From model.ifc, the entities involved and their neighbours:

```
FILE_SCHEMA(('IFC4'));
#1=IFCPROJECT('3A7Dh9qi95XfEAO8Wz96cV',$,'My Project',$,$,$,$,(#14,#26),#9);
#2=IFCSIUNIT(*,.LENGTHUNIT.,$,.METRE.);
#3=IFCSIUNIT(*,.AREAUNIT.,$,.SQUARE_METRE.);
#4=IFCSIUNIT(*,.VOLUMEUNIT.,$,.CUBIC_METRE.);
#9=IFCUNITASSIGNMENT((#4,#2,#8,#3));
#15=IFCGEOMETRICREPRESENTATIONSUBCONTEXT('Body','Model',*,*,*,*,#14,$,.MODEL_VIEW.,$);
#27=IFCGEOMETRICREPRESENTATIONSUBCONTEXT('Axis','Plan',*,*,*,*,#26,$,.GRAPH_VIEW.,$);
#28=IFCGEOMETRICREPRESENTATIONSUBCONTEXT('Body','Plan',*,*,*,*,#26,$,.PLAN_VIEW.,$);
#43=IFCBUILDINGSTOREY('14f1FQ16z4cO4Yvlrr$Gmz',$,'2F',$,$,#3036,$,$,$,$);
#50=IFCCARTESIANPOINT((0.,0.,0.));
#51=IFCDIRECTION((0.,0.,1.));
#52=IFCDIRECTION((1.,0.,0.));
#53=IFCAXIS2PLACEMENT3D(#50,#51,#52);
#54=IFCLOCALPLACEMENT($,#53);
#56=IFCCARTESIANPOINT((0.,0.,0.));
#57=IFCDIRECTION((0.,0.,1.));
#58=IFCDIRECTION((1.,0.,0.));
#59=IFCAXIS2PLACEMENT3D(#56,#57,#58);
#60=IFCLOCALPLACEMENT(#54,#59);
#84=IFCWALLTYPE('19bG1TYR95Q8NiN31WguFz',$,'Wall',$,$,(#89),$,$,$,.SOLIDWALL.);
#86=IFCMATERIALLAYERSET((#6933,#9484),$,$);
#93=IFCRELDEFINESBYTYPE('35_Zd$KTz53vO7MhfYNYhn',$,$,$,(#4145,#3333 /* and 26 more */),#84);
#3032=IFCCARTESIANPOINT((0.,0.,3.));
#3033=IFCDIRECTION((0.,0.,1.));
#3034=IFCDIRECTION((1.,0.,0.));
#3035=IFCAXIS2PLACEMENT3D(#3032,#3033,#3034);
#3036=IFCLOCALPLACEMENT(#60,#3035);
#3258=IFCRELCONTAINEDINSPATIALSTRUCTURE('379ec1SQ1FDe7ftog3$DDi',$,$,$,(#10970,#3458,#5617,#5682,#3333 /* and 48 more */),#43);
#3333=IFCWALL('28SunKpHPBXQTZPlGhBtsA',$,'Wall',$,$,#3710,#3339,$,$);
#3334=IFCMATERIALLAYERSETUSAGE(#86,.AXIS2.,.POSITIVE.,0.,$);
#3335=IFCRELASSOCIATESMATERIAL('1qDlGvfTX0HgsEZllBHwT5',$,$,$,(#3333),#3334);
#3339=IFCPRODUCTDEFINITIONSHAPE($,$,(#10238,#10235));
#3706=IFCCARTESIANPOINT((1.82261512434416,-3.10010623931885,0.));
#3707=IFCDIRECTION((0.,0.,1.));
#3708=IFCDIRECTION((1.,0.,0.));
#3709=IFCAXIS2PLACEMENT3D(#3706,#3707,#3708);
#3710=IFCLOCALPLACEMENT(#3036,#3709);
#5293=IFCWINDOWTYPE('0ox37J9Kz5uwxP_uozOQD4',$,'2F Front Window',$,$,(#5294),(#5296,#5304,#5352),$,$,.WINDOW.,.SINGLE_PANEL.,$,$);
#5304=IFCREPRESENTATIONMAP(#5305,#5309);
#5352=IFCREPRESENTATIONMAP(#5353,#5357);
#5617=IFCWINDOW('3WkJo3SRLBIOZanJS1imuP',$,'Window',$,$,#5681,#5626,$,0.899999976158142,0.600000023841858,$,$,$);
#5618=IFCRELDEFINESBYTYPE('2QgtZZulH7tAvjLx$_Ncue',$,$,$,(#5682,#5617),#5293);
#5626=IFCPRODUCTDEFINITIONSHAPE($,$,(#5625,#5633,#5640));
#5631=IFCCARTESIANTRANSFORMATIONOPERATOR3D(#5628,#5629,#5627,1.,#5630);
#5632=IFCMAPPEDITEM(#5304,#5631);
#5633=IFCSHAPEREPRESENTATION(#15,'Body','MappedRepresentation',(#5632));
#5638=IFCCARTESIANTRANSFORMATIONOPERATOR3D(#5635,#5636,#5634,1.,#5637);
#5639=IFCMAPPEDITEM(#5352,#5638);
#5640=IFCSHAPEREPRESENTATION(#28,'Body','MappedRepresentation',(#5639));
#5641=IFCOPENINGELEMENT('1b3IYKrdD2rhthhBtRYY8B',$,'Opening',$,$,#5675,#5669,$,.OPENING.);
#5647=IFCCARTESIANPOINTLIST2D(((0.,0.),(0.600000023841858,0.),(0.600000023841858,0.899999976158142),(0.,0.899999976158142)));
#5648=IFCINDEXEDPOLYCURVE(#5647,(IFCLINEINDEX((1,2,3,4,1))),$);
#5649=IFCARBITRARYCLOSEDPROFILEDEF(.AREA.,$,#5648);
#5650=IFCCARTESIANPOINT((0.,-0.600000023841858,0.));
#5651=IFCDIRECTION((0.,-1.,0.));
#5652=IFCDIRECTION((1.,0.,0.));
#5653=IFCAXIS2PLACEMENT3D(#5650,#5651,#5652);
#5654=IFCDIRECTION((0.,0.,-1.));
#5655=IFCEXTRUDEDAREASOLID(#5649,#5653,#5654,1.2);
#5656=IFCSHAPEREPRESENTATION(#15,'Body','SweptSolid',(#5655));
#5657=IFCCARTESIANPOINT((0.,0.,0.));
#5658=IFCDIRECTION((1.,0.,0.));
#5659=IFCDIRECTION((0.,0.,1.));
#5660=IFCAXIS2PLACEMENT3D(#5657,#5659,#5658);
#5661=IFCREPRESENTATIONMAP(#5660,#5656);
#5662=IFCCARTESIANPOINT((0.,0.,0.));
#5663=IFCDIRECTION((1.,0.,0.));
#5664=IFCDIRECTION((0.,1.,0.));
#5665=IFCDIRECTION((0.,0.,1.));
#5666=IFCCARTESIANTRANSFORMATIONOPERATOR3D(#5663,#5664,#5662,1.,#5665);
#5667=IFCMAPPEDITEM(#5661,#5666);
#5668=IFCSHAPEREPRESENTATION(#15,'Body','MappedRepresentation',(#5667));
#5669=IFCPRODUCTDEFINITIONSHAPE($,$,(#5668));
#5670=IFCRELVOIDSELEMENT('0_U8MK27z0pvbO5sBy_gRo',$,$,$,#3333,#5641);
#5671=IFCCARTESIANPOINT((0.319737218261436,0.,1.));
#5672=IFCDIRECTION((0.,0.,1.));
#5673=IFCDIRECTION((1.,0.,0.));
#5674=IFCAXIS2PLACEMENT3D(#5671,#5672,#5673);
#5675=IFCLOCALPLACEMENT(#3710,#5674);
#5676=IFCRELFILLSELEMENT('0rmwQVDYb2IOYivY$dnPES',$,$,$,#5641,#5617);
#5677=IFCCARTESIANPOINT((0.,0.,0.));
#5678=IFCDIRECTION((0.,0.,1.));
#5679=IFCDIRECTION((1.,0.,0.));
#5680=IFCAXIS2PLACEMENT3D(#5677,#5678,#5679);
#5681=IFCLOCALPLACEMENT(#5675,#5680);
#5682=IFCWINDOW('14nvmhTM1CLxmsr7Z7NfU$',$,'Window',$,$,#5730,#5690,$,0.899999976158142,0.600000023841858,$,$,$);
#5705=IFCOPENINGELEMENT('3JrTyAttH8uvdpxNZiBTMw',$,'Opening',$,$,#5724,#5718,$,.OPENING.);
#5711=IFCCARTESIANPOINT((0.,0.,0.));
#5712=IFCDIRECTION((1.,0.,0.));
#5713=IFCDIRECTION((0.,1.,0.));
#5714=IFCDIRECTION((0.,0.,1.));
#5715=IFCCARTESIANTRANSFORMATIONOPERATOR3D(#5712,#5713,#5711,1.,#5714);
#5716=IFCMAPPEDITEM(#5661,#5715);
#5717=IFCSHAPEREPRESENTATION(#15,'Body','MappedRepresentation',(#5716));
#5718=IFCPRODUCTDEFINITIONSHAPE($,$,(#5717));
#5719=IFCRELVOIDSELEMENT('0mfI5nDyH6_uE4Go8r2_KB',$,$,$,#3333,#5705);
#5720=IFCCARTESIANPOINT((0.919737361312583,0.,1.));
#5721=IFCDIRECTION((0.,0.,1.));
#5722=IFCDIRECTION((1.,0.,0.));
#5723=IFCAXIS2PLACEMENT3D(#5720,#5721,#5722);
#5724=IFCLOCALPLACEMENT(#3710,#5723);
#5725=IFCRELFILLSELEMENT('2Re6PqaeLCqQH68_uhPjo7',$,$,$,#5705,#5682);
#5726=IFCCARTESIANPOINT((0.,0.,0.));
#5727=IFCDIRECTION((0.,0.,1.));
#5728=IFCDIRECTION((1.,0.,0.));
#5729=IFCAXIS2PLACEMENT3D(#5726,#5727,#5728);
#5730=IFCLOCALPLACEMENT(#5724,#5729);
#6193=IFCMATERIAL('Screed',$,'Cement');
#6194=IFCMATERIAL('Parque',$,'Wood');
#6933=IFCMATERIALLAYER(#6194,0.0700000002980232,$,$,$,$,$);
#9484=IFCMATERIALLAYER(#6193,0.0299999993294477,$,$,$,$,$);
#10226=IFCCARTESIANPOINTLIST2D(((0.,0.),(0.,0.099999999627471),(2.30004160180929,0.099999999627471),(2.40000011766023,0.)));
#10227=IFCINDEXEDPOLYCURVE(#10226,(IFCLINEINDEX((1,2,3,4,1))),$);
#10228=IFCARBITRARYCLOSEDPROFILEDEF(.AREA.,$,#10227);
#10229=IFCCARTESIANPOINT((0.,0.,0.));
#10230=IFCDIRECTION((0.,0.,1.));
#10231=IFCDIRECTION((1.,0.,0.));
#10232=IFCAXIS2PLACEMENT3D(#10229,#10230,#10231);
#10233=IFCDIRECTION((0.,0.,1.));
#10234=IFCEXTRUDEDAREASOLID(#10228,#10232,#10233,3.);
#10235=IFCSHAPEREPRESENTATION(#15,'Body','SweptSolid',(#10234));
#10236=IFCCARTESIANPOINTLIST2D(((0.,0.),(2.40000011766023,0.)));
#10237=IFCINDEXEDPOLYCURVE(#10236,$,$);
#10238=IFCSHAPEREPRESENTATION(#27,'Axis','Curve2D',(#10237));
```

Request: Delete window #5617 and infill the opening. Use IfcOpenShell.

```python
import ifcopenshell
import ifcopenshell.api.feature
import ifcopenshell.api.root
import ifcopenshell.geom
import ifcopenshell.util.shape

model = ifcopenshell.open("model.ifc")
settings = ifcopenshell.geom.settings()


def volume(element):
    """Net volume in cubic metres, openings subtracted."""
    shape = ifcopenshell.geom.create_shape(settings, element)
    return ifcopenshell.util.shape.get_volume(shape.geometry)


window = model.by_guid("3WkJo3SRLBIOZanJS1imuP")
opening = window.FillsVoids[0].RelatingOpeningElement
wall = opening.VoidsElements[0].RelatingBuildingElement
before = volume(wall)

ifcopenshell.api.root.remove_product(model, product=window)
ifcopenshell.api.feature.remove_feature(model, feature=opening)

after = volume(wall)

print(f"wall volume {before:.3f} -> {after:.3f} m3")

model.write("model_updated.ifc")
```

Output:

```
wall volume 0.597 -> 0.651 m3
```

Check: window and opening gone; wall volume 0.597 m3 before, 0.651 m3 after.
